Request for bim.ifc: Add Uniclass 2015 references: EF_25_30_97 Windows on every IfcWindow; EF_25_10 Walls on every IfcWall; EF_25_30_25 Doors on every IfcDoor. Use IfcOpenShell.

First a look at what the model holds.

```python
import ifcopenshell

model = ifcopenshell.open("bim.ifc")
print(model.schema)
print("classifications:", [c.Name for c in model.by_type("IfcClassification")])
for ifc_class in ("IfcDoor", "IfcRoof", "IfcStair", "IfcWall", "IfcWindow"):
    print(ifc_class, len(model.by_type(ifc_class)))
```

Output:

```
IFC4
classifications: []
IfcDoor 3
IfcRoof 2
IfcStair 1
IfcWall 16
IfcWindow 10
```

```python
import ifcopenshell
import ifcopenshell.api.classification

model = ifcopenshell.open("bim.ifc")

system = ifcopenshell.api.classification.add_classification(model, classification="Uniclass 2015")

codes = {
    "IfcWindow": ("EF_25_30_97", "Windows"),
    "IfcWall": ("EF_25_10", "Walls"),
    "IfcDoor": ("EF_25_30_25", "Doors"),
}
for ifc_class, (code, name) in codes.items():
    products = model.by_type(ifc_class)
    ifcopenshell.api.classification.add_reference(
        model, products=products, classification=system, identification=code, name=name
    )
    print(code, len(products))

model.write("bim_v2.ifc")
```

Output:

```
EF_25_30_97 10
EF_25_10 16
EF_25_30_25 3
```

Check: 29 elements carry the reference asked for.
